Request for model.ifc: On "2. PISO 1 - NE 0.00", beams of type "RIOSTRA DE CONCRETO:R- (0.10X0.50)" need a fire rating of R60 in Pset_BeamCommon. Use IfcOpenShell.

First a look at what the model holds.

```python
import ifcopenshell
import ifcopenshell.util.element

model = ifcopenshell.open("model.ifc")
print(model.schema)
storey = next(s for s in model.by_type("IfcBuildingStorey") if s.Name == "2. PISO 1 - NE 0.00")
beams = [e for e in ifcopenshell.util.element.get_decomposition(storey) if e.is_a("IfcBeam")]
seen = {}
for e in beams:
    element_type = ifcopenshell.util.element.get_type(e)
    key = (element_type.Name if element_type != e and element_type else None, ifcopenshell.util.element.get_pset(e, "Pset_BeamCommon", "FireRating"))
    seen[key] = seen.get(key, 0) + 1
for (name, value), count in sorted(seen.items(), key=str):
    print(count, "x", name, "|", value)
```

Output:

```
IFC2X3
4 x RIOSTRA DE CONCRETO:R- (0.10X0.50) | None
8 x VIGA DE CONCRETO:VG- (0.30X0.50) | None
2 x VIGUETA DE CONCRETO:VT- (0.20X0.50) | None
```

```python
import ifcopenshell
import ifcopenshell.api.pset
import ifcopenshell.util.element

model = ifcopenshell.open("model.ifc")

storey = next(s for s in model.by_type("IfcBuildingStorey") if s.Name == "2. PISO 1 - NE 0.00")
beams = [e for e in ifcopenshell.util.element.get_decomposition(storey) if e.is_a("IfcBeam")]

count = 0
for e in beams:
    element_type = ifcopenshell.util.element.get_type(e)
    if element_type in (None, e) or element_type.Name != "RIOSTRA DE CONCRETO:R- (0.10X0.50)":
        continue
    # add_pset returns the element's existing set when there is one.
    pset = ifcopenshell.api.pset.add_pset(model, product=e, name="Pset_BeamCommon")
    ifcopenshell.api.pset.edit_pset(model, pset=pset, properties={"FireRating": "R60"})
    count += 1

print(count, "beams updated")

model.write("model_updated.ifc")
```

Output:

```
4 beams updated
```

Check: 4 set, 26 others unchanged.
